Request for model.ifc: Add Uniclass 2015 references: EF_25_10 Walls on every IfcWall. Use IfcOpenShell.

First a look at what the model holds.

```python
import ifcopenshell

model = ifcopenshell.open("model.ifc")
print(model.schema)
print("classifications:", [c.Name for c in model.by_type("IfcClassification")])
for ifc_class in ("IfcDoor", "IfcRoof", "IfcStair", "IfcWall", "IfcWindow"):
    print(ifc_class, len(model.by_type(ifc_class)))
```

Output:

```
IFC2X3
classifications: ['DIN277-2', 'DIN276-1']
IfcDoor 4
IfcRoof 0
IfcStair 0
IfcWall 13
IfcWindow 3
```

```python
import ifcopenshell
import ifcopenshell.api.classification

model = ifcopenshell.open("model.ifc")

# IFC2X3 requires Source and Edition and has no link from the project to the system.
system = model.create_entity("IfcClassification", Source="NBS", Edition="2015", Name="Uniclass 2015")

codes = {
    "IfcWall": ("EF_25_10", "Walls"),
}
for ifc_class, (code, name) in codes.items():
    products = model.by_type(ifc_class)
    ifcopenshell.api.classification.add_reference(
        model, products=products, classification=system, identification=code, name=name
    )
    print(code, len(products))

model.write("model_updated.ifc")
```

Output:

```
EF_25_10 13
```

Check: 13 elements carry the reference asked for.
